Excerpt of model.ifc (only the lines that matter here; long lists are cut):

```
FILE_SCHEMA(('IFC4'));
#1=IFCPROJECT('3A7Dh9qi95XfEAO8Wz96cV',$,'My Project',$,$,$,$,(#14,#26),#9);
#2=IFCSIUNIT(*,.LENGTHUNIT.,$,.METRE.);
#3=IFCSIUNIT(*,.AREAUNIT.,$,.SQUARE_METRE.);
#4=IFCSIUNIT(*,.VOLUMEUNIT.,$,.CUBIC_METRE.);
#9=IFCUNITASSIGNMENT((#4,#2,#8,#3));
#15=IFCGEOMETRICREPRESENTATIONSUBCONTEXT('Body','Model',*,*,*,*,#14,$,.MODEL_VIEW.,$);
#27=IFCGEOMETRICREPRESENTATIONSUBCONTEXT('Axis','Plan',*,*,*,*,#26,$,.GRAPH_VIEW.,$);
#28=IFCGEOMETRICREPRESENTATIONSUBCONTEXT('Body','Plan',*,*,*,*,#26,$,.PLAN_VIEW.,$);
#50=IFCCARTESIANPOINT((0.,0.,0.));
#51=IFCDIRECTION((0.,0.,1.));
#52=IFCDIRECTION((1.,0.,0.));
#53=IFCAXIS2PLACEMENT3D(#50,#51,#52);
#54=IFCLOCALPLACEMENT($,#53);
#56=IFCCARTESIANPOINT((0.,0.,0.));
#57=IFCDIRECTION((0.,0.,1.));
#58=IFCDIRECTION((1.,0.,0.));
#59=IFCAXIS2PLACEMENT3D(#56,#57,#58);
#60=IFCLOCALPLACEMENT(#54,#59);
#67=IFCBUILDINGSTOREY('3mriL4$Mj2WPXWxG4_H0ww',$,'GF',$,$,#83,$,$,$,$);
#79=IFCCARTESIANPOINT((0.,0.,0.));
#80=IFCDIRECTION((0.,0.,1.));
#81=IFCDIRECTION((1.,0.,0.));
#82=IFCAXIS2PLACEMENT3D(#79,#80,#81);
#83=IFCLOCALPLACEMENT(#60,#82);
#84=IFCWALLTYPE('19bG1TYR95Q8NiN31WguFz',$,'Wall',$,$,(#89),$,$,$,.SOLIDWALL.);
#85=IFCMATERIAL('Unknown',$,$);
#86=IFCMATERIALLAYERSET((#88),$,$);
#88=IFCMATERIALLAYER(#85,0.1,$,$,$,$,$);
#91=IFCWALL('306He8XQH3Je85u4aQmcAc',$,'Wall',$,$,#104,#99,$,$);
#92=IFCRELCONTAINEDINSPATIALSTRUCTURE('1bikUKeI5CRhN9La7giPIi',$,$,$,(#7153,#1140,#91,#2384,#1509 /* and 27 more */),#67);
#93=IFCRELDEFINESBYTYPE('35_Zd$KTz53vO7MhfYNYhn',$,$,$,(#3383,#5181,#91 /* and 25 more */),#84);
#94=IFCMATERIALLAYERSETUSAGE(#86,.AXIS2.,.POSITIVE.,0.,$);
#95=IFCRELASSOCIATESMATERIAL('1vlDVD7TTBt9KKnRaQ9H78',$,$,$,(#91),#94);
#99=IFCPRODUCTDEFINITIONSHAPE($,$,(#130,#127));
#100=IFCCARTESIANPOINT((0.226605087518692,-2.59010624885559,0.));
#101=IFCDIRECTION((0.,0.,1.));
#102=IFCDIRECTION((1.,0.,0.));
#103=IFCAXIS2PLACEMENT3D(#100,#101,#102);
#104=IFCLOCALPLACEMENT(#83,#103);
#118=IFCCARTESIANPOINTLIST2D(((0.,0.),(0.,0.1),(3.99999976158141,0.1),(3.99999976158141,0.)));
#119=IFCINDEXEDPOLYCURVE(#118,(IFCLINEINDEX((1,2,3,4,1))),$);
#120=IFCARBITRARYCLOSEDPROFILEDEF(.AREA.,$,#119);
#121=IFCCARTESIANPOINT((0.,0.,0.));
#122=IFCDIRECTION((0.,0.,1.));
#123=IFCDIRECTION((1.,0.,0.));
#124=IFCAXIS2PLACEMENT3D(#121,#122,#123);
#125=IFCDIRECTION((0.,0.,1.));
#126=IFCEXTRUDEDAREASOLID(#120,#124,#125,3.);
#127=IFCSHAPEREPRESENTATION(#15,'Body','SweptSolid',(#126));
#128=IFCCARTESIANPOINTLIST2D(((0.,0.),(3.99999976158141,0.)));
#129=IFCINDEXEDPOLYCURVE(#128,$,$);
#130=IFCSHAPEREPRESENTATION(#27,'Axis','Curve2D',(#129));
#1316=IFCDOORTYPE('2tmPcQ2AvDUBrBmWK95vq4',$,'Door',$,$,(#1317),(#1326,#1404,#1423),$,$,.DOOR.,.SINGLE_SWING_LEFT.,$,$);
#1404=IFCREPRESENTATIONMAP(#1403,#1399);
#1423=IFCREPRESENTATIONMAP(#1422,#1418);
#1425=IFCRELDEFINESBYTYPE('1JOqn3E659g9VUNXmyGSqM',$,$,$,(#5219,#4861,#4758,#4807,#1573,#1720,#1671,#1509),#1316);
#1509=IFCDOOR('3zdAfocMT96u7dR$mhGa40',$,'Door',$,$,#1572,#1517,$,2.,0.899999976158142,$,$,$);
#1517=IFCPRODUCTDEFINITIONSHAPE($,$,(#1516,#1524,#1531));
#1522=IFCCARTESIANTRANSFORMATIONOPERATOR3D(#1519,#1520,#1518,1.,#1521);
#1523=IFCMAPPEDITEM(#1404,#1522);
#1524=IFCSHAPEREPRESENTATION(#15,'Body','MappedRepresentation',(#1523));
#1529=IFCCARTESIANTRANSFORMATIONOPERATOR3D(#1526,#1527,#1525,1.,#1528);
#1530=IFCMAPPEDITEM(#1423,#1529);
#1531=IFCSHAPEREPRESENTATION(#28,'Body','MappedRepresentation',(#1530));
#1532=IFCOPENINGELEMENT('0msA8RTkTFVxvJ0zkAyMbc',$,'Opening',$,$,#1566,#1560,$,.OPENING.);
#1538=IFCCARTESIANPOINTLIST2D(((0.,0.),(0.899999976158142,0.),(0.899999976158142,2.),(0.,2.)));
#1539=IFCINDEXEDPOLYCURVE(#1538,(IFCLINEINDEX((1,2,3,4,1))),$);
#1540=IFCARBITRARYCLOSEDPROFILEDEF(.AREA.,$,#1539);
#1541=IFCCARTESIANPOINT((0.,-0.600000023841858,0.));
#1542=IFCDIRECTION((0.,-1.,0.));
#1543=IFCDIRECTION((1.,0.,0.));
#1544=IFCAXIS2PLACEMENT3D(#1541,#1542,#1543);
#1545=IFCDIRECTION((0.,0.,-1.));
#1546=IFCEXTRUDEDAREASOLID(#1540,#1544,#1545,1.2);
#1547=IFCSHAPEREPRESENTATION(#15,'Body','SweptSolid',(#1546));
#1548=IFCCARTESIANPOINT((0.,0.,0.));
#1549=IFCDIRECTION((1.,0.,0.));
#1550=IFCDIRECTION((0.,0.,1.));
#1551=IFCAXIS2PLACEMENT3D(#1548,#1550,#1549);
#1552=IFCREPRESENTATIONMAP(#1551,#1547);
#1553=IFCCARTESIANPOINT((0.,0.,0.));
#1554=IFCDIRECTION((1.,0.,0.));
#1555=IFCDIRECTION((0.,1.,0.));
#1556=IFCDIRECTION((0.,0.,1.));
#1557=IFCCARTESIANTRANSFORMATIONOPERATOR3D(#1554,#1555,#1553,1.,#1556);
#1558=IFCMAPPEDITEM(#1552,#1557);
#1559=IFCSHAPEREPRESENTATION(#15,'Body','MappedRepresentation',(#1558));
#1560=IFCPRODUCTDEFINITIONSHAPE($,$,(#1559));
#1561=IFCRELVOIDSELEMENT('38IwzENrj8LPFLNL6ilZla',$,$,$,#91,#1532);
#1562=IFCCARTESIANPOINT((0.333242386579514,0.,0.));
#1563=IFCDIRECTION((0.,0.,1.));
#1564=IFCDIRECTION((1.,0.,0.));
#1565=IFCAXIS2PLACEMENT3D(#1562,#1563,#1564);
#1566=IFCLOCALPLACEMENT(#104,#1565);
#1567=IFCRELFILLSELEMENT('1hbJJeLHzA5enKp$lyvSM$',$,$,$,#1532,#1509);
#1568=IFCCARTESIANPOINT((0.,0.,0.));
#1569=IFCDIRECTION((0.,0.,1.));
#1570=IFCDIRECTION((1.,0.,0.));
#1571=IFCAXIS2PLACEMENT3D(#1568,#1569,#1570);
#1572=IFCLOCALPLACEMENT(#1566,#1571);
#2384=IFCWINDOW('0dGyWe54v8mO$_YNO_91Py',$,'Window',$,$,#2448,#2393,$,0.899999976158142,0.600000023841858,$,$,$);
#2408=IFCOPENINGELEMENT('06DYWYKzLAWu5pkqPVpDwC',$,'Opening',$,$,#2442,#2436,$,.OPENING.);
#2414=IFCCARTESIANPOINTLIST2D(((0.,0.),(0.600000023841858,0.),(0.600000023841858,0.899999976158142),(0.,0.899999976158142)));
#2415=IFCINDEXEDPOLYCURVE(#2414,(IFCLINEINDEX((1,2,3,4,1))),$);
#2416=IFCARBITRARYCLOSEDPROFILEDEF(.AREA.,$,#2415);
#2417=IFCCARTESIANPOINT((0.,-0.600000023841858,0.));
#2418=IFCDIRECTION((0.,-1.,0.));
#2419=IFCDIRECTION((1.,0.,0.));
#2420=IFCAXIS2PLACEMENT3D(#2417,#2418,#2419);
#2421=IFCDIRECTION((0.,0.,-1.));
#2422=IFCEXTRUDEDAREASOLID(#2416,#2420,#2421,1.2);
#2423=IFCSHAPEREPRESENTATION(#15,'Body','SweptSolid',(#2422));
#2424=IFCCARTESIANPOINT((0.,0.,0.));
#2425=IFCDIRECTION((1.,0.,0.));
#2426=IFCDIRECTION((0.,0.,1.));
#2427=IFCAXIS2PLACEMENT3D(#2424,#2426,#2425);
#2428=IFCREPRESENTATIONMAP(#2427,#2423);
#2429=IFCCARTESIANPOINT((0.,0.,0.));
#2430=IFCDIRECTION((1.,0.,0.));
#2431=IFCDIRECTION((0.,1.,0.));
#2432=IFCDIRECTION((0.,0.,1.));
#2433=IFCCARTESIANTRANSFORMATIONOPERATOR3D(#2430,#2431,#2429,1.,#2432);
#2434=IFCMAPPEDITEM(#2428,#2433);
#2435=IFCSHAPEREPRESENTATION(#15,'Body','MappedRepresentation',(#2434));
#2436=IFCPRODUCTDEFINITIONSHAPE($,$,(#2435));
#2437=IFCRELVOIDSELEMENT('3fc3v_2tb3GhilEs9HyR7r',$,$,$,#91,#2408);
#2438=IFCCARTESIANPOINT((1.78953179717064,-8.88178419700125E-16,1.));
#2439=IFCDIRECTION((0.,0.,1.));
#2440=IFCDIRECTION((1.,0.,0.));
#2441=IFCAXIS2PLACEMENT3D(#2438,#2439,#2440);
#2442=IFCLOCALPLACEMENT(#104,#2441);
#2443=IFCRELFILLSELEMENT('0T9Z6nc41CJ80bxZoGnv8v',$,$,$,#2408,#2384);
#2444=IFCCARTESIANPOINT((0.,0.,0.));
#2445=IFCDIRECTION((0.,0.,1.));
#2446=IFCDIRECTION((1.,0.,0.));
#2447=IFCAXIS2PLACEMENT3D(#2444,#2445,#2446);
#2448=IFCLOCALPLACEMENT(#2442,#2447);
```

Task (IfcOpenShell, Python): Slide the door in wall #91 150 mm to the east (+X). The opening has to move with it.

```python
import ifcopenshell
import ifcopenshell.api.geometry
import ifcopenshell.util.placement
import ifcopenshell.util.unit

model = ifcopenshell.open("model.ifc")
unit_scale = ifcopenshell.util.unit.calculate_unit_scale(model)

door = model.by_id(1509)
opening = door.FillsVoids[0].RelatingOpeningElement
wall = opening.VoidsElements[0].RelatingBuildingElement

wall_matrix = ifcopenshell.util.placement.get_local_placement(wall.ObjectPlacement)
shift = wall_matrix[:3, 0] * 0.15 / unit_scale
before = ifcopenshell.util.placement.get_local_placement(door.ObjectPlacement)[:3, 3].copy()

# The door is placed relative to its opening, so it follows when the opening moves.
matrix = ifcopenshell.util.placement.get_local_placement(opening.ObjectPlacement)
matrix[:3, 3] += shift
ifcopenshell.api.geometry.edit_object_placement(
    model, product=opening, matrix=matrix, is_si=False, should_transform_children=True
)

after = ifcopenshell.util.placement.get_local_placement(door.ObjectPlacement)[:3, 3]
print("door moved by", (after - before).round(3) + 0.0)

model.write("model_v2.ifc")
```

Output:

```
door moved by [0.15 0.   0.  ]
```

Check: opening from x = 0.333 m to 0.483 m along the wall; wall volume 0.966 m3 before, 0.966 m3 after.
